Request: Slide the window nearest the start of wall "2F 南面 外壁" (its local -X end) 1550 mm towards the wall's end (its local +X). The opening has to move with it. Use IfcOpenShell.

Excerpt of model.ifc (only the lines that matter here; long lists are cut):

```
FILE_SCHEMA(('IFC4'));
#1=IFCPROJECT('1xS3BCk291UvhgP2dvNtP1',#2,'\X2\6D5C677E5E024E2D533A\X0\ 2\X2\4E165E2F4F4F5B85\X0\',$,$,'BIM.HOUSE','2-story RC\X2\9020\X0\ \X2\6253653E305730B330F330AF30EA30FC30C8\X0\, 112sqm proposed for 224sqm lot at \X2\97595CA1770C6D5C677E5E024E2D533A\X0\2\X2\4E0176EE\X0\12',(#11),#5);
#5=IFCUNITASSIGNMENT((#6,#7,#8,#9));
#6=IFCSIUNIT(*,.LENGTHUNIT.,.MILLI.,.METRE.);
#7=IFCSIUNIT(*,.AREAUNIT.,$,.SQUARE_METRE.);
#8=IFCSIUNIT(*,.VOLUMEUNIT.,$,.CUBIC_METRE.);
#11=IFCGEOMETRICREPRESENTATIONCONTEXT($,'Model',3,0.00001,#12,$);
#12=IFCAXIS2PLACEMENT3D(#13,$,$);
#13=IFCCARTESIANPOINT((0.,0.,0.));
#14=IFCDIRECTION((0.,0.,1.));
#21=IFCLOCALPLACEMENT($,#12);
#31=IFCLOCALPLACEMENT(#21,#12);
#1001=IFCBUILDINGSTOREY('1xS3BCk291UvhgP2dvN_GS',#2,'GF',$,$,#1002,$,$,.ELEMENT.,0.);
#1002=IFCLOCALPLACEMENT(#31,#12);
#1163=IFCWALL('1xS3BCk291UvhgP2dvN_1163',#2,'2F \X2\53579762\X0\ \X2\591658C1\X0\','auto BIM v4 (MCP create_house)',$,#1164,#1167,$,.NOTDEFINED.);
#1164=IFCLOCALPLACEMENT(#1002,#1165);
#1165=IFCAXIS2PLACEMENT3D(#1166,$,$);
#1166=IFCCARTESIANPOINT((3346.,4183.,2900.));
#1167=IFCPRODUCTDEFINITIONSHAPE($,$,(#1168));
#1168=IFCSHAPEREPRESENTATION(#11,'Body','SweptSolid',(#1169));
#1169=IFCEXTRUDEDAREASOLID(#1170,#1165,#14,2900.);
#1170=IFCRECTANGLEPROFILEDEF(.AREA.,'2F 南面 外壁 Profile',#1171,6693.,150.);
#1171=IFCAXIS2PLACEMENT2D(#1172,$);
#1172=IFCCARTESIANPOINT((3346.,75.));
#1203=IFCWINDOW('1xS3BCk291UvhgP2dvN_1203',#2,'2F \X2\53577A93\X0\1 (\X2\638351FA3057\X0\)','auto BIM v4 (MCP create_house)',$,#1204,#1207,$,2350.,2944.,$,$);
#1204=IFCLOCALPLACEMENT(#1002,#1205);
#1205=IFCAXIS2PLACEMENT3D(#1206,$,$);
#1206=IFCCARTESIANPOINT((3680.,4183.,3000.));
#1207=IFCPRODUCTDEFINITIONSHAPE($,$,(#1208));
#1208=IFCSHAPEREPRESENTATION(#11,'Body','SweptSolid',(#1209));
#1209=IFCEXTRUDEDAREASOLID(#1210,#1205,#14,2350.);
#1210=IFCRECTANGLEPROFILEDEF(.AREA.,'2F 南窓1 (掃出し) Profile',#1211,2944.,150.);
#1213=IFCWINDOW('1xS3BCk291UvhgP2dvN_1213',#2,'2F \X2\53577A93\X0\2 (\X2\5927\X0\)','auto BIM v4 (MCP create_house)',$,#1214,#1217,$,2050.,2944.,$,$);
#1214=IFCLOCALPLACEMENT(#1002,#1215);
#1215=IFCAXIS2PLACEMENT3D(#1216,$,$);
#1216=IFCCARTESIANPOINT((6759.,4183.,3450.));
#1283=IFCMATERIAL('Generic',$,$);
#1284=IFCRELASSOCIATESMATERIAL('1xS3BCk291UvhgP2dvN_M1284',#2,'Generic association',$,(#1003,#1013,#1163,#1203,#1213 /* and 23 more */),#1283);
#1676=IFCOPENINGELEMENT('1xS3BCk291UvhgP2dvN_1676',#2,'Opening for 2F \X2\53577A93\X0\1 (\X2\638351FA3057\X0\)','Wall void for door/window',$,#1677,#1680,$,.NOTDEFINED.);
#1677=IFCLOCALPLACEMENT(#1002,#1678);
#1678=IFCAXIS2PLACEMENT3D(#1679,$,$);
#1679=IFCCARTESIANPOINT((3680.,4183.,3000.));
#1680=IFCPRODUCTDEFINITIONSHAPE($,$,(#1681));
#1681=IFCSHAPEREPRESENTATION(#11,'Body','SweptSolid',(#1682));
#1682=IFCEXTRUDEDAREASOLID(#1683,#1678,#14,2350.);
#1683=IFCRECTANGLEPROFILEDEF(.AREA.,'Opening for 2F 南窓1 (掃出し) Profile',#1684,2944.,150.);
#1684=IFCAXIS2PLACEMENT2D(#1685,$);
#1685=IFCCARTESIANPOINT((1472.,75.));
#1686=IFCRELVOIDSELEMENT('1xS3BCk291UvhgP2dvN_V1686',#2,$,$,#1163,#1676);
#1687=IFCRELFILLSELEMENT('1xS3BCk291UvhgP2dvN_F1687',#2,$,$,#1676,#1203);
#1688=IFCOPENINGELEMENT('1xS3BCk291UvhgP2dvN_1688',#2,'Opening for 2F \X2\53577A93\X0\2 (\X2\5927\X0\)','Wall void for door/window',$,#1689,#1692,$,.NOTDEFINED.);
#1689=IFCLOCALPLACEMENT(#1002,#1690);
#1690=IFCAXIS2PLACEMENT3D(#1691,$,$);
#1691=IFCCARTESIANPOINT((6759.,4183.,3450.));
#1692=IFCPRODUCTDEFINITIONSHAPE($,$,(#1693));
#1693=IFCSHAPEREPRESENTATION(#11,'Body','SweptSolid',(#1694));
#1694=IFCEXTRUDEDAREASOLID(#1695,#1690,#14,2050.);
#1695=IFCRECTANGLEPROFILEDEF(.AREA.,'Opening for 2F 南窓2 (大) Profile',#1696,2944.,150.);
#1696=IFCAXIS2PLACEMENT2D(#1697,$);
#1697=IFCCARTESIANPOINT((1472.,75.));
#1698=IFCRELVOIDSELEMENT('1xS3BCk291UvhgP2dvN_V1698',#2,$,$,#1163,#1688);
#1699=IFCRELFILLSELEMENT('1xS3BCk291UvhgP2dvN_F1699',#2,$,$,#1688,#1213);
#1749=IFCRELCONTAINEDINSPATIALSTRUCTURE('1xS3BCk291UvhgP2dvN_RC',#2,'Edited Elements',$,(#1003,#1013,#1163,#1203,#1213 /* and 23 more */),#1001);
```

```python
import ifcopenshell
import ifcopenshell.api.geometry
import ifcopenshell.util.placement
import ifcopenshell.util.unit

model = ifcopenshell.open("model.ifc")
unit_scale = ifcopenshell.util.unit.calculate_unit_scale(model)

window = model.by_guid("1xS3BCk291UvhgP2dvN_1203")
opening = window.FillsVoids[0].RelatingOpeningElement
wall = opening.VoidsElements[0].RelatingBuildingElement

wall_matrix = ifcopenshell.util.placement.get_local_placement(wall.ObjectPlacement)
shift = wall_matrix[:3, 0] * 1.55 / unit_scale
before = ifcopenshell.util.placement.get_local_placement(window.ObjectPlacement)[:3, 3].copy()

# The window is not placed relative to its opening, so move both.
for product in (opening, window):
    matrix = ifcopenshell.util.placement.get_local_placement(product.ObjectPlacement)
    matrix[:3, 3] += shift
    ifcopenshell.api.geometry.edit_object_placement(model, product=product, matrix=matrix, is_si=False)

after = ifcopenshell.util.placement.get_local_placement(window.ObjectPlacement)[:3, 3]
print("window moved by", (after - before).round(3) + 0.0)

model.write("model_v2.ifc")
```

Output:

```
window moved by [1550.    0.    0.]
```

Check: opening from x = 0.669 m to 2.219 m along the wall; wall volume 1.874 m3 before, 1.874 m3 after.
